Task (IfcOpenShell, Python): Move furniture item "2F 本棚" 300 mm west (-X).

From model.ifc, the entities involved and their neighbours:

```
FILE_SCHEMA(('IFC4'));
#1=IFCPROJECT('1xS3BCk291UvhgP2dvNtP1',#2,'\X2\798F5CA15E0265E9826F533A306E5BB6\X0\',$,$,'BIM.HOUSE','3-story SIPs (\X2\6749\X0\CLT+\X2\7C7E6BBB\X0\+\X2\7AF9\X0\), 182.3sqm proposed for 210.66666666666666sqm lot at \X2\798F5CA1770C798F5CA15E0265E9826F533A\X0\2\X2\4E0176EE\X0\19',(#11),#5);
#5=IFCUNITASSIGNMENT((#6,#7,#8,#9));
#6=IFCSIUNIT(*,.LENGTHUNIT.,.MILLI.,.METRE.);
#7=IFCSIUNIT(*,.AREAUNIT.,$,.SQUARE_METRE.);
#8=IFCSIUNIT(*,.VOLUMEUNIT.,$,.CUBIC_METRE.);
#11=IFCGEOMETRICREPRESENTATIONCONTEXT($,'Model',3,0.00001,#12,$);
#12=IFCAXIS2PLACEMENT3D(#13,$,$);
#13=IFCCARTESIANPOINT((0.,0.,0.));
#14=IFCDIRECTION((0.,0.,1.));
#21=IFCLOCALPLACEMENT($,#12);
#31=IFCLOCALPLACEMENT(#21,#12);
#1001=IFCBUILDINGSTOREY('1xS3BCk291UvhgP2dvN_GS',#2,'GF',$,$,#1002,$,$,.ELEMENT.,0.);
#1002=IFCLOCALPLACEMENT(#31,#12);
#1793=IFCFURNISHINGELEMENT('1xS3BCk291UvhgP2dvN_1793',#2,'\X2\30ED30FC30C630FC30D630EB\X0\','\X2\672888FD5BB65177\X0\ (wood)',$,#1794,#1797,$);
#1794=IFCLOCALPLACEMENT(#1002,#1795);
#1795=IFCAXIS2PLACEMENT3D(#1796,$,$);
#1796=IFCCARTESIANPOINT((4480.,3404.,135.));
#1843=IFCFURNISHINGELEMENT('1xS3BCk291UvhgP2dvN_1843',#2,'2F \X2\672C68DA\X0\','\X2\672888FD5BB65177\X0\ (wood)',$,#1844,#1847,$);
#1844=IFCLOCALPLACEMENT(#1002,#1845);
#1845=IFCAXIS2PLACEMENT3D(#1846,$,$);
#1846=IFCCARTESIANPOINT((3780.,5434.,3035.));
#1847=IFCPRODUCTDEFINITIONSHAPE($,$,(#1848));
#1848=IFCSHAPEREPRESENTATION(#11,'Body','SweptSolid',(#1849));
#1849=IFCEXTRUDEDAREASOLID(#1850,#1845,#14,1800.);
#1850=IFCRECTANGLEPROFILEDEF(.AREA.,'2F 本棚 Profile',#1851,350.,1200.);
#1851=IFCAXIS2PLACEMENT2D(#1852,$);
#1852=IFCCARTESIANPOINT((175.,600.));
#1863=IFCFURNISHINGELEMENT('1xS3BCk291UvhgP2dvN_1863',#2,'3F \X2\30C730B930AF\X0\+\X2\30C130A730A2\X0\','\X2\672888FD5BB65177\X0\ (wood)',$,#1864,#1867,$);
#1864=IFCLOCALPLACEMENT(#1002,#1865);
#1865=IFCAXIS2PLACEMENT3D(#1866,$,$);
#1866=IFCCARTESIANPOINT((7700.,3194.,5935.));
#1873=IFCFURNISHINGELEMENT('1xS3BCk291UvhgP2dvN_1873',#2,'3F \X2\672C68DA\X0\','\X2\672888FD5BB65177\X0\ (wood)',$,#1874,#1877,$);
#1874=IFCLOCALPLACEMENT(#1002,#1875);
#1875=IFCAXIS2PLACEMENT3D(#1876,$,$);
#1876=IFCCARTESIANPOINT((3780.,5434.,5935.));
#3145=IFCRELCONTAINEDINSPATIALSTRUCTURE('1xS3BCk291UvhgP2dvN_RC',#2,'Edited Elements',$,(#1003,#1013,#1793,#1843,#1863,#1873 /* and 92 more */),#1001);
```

```python
import ifcopenshell
import ifcopenshell.api.geometry
import ifcopenshell.util.placement

model = ifcopenshell.open("model.ifc")

item = model.by_guid("1xS3BCk291UvhgP2dvN_1843")
matrix = ifcopenshell.util.placement.get_local_placement(item.ObjectPlacement)
matrix[0, 3] -= 300.0
ifcopenshell.api.geometry.edit_object_placement(model, product=item, matrix=matrix, is_si=False)

print(ifcopenshell.util.placement.get_local_placement(item.ObjectPlacement).round(3) + 0.0)

model.write("model_v2.ifc")
```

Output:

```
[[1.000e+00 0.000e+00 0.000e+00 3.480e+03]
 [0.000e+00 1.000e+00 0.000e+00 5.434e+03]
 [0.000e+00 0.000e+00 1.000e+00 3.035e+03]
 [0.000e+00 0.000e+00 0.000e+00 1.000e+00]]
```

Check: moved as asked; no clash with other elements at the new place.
